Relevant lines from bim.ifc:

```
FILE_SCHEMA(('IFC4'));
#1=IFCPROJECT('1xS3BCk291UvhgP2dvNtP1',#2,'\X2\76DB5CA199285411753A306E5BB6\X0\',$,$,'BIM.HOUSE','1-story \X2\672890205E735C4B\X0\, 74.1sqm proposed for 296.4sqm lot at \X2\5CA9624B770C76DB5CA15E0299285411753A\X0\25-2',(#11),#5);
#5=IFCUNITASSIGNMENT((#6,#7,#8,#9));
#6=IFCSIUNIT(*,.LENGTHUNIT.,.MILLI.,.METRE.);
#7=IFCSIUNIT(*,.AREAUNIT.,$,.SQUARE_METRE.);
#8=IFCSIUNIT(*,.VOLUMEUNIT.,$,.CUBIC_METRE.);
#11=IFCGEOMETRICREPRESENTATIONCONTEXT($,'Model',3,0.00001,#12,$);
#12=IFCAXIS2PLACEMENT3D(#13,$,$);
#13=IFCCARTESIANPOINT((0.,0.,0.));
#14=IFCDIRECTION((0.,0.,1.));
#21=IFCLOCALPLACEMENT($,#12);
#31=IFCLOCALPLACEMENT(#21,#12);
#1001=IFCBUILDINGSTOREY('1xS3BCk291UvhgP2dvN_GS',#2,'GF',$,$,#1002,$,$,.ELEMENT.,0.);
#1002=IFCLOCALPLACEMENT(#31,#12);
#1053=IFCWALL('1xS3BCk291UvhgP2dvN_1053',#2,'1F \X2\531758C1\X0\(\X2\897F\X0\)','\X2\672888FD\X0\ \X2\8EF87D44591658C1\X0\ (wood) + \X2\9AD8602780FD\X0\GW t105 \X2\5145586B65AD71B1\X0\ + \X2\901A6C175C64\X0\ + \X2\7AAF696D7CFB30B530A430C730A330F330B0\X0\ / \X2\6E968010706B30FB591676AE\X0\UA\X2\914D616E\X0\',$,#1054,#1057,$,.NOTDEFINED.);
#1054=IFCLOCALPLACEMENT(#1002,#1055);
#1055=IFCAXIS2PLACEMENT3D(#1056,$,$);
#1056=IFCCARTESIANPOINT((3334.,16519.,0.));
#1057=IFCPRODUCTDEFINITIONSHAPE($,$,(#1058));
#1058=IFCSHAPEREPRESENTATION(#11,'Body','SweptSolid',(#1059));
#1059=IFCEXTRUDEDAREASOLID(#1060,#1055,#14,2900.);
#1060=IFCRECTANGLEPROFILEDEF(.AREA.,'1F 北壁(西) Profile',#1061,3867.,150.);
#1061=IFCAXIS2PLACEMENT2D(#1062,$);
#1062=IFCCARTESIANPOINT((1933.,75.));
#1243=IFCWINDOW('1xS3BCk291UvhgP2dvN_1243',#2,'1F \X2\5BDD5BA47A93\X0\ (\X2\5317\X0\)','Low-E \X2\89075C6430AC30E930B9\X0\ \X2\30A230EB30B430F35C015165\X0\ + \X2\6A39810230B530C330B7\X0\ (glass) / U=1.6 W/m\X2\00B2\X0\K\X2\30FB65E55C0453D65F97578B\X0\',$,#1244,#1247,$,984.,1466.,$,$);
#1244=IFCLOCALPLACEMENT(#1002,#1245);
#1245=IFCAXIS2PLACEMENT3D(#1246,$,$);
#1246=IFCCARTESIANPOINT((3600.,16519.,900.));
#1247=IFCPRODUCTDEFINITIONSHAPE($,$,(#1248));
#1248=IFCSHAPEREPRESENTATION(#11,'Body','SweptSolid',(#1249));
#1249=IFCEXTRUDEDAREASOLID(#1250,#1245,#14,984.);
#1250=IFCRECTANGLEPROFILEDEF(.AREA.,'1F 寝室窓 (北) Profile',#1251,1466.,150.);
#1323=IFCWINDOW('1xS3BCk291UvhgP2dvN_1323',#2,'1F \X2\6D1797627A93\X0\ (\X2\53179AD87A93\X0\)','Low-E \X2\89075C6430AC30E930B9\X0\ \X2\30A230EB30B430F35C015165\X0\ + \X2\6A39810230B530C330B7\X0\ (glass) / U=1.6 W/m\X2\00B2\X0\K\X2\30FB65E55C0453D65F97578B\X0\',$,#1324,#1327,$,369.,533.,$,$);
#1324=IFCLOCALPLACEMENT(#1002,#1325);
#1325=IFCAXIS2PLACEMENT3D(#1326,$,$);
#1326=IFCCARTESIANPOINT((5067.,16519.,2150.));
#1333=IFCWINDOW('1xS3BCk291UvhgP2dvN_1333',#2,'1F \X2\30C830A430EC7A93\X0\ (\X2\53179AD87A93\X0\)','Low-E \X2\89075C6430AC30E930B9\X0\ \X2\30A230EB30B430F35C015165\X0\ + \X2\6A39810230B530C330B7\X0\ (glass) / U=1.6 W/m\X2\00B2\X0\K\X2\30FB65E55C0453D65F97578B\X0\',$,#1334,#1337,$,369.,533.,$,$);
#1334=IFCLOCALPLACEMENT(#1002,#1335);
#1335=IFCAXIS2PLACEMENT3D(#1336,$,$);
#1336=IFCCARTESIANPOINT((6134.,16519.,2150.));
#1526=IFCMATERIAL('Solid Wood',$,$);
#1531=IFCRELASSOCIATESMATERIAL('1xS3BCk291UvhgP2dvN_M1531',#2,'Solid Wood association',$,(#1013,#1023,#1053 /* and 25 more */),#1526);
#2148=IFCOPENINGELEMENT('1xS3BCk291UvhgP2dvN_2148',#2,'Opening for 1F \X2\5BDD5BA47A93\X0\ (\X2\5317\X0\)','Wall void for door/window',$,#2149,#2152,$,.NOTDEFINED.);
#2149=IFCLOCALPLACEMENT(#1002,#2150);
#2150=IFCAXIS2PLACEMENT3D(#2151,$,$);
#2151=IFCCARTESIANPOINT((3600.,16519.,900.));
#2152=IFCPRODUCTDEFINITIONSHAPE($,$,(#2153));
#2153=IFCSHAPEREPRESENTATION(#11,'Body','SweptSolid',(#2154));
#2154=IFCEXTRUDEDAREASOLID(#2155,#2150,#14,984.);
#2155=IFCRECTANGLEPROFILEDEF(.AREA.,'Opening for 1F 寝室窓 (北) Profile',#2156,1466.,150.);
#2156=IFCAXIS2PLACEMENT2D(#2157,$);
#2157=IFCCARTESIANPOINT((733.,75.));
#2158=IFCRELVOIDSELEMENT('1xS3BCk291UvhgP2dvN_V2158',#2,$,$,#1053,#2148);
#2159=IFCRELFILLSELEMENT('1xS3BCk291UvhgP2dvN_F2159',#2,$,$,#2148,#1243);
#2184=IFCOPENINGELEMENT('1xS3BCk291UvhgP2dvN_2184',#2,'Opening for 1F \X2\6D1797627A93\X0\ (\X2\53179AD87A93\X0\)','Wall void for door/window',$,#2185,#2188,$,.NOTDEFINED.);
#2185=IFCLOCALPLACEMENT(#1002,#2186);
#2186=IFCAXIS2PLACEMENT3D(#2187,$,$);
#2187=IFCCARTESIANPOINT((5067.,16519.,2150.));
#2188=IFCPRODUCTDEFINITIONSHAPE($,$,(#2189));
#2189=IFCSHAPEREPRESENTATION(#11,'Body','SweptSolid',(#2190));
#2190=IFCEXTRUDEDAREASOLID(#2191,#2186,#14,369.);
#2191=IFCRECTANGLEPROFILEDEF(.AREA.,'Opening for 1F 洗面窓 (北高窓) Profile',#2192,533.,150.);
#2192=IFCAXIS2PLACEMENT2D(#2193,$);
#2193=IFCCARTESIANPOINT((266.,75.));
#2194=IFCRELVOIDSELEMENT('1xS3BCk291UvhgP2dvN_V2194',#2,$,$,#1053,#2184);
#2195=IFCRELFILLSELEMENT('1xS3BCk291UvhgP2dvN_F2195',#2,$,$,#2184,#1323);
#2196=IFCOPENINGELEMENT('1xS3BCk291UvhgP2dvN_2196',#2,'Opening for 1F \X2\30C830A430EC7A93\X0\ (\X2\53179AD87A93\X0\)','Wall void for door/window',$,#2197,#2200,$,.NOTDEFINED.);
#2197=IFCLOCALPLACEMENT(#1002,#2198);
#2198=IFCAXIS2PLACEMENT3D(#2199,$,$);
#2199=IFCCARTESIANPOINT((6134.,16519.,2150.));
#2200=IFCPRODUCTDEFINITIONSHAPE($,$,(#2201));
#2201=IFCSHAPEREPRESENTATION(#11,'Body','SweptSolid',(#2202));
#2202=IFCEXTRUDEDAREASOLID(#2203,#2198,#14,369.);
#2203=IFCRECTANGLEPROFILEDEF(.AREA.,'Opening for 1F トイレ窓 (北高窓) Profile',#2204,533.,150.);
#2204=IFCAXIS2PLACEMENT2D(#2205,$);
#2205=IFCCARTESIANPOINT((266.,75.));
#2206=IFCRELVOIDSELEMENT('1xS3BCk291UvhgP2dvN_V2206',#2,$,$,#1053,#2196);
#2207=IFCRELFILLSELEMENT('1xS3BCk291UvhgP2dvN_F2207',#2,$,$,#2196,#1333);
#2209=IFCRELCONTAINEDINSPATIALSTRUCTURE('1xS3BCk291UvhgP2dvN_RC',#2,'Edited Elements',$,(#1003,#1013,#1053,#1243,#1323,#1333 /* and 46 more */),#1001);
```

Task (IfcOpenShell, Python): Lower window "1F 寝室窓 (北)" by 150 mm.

```python
import numpy as np
import ifcopenshell
import ifcopenshell.api.geometry
import ifcopenshell.util.placement
import ifcopenshell.util.unit

model = ifcopenshell.open("bim.ifc")
unit_scale = ifcopenshell.util.unit.calculate_unit_scale(model)

window = model.by_guid("1xS3BCk291UvhgP2dvN_1243")
opening = window.FillsVoids[0].RelatingOpeningElement
dz = -0.15 / unit_scale

shift = np.array([0.0, 0.0, dz])
# The window is not placed relative to its opening, so move both.
for product in (opening, window):
    matrix = ifcopenshell.util.placement.get_local_placement(product.ObjectPlacement)
    matrix[:3, 3] += shift
    ifcopenshell.api.geometry.edit_object_placement(model, product=product, matrix=matrix, is_si=False)

print(f"moved by {dz * unit_scale:+.3f} m")

model.write("bim-out.ifc")
```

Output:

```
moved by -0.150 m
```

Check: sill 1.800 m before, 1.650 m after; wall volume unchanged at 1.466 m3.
